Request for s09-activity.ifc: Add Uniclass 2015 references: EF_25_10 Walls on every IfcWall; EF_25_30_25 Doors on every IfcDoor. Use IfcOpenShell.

First a look at what the model holds.

```python
import ifcopenshell

model = ifcopenshell.open("s09-activity.ifc")
print(model.schema)
print("classifications:", [c.Name for c in model.by_type("IfcClassification")])
for ifc_class in ("IfcDoor", "IfcRoof", "IfcStair", "IfcWall", "IfcWindow"):
    print(ifc_class, len(model.by_type(ifc_class)))
```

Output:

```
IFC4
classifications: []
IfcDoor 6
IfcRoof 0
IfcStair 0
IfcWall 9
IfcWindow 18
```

```python
import ifcopenshell
import ifcopenshell.api.classification

model = ifcopenshell.open("s09-activity.ifc")

system = ifcopenshell.api.classification.add_classification(model, classification="Uniclass 2015")

codes = {
    "IfcWall": ("EF_25_10", "Walls"),
    "IfcDoor": ("EF_25_30_25", "Doors"),
}
for ifc_class, (code, name) in codes.items():
    products = model.by_type(ifc_class)
    ifcopenshell.api.classification.add_reference(
        model, products=products, classification=system, identification=code, name=name
    )
    print(code, len(products))

model.write("s09-activity_edited.ifc")
```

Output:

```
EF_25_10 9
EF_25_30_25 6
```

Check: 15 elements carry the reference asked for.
